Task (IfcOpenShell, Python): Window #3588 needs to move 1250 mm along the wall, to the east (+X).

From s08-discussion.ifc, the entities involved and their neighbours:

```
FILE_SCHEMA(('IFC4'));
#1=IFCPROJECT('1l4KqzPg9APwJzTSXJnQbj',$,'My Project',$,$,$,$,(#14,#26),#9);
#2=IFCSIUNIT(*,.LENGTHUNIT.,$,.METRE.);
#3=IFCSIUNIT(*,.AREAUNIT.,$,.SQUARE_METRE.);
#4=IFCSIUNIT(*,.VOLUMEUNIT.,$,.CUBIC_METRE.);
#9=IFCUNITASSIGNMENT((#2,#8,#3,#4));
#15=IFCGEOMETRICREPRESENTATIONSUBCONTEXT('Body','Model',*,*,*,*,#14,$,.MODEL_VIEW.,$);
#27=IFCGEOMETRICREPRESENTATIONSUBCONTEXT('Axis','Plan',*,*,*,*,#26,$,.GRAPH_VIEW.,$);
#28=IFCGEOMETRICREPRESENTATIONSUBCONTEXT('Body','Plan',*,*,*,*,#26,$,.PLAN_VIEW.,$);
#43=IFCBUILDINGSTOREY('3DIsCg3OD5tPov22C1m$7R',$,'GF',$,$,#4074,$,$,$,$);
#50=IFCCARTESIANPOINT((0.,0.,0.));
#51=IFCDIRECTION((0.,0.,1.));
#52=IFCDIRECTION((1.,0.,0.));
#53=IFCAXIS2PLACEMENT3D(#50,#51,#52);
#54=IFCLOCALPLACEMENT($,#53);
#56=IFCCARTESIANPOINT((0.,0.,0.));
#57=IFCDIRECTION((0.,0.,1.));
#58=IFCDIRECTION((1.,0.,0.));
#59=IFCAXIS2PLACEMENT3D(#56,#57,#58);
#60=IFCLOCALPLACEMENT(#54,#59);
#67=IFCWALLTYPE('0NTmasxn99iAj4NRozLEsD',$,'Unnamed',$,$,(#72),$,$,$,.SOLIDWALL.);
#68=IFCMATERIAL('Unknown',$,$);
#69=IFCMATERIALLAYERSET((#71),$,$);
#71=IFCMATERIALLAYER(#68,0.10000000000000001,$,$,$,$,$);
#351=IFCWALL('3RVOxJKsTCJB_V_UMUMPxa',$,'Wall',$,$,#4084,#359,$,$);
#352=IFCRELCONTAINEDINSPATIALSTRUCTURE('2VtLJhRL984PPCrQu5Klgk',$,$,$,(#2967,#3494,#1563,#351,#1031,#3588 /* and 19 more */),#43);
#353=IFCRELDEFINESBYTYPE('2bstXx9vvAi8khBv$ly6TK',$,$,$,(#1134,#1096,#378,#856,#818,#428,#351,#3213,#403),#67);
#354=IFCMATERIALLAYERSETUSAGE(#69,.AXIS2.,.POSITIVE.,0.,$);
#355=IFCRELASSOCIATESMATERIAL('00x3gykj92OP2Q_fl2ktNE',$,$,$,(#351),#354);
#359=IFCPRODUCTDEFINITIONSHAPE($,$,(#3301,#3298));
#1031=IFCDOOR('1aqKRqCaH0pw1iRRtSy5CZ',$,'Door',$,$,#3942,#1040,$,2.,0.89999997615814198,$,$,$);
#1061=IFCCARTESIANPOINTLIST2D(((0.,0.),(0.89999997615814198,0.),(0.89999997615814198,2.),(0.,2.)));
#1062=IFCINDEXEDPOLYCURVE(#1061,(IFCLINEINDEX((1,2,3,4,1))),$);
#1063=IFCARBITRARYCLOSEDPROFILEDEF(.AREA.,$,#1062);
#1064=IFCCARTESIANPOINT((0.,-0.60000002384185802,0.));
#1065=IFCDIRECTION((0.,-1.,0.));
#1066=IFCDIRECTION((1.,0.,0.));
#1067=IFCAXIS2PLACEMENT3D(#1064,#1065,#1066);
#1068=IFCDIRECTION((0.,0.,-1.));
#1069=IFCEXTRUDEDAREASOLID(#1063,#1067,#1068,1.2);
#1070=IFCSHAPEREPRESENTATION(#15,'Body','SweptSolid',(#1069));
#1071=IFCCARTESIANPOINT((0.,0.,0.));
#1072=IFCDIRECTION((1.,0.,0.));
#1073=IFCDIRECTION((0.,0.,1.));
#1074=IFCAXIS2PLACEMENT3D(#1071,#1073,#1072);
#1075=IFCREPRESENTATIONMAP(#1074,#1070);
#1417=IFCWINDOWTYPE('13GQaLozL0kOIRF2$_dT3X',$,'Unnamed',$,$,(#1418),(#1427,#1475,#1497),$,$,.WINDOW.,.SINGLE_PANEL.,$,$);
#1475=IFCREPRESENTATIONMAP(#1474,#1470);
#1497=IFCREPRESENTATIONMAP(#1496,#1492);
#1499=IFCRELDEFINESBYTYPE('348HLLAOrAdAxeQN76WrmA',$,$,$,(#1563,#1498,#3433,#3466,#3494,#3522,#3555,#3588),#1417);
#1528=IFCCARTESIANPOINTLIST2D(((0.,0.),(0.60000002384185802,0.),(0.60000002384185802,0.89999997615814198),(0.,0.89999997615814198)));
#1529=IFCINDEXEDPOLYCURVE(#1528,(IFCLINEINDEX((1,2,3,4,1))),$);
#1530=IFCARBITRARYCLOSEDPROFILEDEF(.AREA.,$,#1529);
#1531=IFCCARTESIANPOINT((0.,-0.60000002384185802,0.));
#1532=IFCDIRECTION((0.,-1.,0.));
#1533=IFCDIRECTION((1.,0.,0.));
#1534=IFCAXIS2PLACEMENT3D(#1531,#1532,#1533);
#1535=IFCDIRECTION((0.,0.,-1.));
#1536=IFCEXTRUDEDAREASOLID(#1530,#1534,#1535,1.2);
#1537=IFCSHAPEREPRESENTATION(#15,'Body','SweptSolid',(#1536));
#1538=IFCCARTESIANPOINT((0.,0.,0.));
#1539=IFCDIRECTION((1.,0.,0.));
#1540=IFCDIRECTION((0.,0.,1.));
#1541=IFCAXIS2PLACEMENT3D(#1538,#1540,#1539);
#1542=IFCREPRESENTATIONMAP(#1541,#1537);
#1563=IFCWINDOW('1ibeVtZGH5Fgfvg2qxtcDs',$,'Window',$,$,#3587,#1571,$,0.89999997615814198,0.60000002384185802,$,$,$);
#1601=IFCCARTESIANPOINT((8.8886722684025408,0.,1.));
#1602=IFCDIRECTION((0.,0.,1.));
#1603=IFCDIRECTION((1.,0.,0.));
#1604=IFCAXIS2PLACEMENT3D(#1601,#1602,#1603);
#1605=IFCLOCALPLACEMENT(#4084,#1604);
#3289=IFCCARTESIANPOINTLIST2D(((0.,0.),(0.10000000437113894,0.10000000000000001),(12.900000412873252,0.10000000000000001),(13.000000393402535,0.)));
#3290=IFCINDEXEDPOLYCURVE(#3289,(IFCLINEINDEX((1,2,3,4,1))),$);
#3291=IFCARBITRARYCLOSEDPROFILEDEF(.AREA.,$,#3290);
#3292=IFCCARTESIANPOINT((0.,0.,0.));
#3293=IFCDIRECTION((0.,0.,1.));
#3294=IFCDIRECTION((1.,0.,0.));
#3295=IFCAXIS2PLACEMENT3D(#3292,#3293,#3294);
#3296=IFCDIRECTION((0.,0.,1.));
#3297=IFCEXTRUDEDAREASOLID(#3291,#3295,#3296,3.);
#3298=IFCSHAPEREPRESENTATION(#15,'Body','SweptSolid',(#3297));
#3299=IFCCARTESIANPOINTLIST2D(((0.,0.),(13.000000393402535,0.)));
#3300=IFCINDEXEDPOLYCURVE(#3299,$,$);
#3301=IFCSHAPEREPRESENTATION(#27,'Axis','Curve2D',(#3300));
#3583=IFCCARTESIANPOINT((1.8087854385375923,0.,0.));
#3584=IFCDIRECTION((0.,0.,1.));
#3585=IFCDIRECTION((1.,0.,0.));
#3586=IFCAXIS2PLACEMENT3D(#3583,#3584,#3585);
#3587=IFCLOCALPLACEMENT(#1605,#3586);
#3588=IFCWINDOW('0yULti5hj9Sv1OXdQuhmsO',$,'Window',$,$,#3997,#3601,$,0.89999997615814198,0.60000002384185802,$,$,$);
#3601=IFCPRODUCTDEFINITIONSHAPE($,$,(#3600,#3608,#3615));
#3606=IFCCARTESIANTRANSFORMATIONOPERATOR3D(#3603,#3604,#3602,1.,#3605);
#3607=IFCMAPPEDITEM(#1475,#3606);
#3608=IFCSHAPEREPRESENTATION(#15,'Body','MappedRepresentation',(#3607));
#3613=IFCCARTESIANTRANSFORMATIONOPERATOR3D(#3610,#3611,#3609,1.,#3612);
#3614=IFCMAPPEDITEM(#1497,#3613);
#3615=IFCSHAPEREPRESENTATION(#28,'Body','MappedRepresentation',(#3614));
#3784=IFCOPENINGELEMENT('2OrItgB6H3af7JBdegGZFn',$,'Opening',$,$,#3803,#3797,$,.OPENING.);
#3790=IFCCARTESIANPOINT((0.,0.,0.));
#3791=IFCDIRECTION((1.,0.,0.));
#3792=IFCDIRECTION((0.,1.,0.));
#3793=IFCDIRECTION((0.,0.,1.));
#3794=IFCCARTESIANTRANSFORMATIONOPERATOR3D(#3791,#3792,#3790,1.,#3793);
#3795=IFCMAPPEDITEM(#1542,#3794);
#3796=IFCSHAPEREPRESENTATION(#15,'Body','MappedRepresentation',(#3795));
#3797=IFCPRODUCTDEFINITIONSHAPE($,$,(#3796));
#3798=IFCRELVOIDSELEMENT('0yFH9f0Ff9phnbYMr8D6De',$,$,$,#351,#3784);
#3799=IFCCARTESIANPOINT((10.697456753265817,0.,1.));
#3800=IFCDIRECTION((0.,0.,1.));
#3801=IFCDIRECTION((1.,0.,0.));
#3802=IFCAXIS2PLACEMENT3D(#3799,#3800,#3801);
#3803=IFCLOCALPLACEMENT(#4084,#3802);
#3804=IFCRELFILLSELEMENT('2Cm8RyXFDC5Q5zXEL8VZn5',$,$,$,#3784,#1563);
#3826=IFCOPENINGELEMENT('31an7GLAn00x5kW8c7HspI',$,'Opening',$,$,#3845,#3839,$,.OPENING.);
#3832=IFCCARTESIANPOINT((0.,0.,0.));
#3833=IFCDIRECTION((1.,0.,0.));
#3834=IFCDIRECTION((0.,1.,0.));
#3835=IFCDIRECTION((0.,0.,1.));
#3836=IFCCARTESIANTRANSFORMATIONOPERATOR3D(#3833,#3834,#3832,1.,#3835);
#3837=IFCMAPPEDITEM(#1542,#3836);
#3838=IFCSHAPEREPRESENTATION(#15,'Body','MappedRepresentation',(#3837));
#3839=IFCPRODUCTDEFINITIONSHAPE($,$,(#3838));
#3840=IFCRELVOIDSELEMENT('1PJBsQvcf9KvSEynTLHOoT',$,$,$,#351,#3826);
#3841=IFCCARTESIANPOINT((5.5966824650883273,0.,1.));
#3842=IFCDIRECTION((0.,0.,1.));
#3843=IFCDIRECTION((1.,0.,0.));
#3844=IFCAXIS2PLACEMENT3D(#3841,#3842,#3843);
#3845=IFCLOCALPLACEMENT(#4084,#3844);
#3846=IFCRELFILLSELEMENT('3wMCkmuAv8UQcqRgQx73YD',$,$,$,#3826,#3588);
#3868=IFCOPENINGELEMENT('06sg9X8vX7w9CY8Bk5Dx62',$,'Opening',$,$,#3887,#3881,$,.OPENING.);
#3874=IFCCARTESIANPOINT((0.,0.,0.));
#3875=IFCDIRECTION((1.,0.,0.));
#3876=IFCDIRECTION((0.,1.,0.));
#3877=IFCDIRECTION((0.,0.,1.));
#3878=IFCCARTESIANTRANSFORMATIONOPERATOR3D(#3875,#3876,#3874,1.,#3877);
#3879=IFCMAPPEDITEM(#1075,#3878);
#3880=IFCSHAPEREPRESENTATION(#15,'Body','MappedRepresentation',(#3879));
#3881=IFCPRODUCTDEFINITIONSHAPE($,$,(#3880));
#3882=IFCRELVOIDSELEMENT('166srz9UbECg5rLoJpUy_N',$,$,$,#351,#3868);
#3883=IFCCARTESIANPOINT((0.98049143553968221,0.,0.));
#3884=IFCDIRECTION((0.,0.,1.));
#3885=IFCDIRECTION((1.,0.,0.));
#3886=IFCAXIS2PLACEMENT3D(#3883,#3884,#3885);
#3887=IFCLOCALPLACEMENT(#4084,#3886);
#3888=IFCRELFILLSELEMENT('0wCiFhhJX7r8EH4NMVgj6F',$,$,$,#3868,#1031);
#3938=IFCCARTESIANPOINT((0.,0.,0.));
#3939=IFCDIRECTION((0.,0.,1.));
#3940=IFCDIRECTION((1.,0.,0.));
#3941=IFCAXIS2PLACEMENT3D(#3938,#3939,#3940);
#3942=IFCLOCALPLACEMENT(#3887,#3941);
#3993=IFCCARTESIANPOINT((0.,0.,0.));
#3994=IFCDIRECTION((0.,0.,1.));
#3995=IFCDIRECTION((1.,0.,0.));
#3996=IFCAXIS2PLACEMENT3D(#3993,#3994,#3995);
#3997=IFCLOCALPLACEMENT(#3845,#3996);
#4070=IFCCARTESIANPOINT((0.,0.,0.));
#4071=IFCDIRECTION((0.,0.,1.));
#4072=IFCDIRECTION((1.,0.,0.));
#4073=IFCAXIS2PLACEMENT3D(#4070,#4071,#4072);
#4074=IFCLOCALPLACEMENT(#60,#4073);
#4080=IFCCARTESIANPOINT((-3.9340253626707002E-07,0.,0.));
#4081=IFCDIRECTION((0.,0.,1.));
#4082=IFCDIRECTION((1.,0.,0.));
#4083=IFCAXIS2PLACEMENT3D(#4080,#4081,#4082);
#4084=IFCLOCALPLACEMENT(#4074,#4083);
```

```python
import ifcopenshell
import ifcopenshell.api.geometry
import ifcopenshell.util.placement
import ifcopenshell.util.unit

model = ifcopenshell.open("s08-discussion.ifc")
unit_scale = ifcopenshell.util.unit.calculate_unit_scale(model)

window = model.by_guid("0yULti5hj9Sv1OXdQuhmsO")
opening = window.FillsVoids[0].RelatingOpeningElement
wall = opening.VoidsElements[0].RelatingBuildingElement

wall_matrix = ifcopenshell.util.placement.get_local_placement(wall.ObjectPlacement)
shift = wall_matrix[:3, 0] * 1.25 / unit_scale
before = ifcopenshell.util.placement.get_local_placement(window.ObjectPlacement)[:3, 3].copy()

# The window is placed relative to its opening, so it follows when the opening moves.
matrix = ifcopenshell.util.placement.get_local_placement(opening.ObjectPlacement)
matrix[:3, 3] += shift
ifcopenshell.api.geometry.edit_object_placement(
    model, product=opening, matrix=matrix, is_si=False, should_transform_children=True
)

after = ifcopenshell.util.placement.get_local_placement(window.ObjectPlacement)[:3, 3]
print("window moved by", (after - before).round(3) + 0.0)

model.write("s08-discussion-out.ifc")
```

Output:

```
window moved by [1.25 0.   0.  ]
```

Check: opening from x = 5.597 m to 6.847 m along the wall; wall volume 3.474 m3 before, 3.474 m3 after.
